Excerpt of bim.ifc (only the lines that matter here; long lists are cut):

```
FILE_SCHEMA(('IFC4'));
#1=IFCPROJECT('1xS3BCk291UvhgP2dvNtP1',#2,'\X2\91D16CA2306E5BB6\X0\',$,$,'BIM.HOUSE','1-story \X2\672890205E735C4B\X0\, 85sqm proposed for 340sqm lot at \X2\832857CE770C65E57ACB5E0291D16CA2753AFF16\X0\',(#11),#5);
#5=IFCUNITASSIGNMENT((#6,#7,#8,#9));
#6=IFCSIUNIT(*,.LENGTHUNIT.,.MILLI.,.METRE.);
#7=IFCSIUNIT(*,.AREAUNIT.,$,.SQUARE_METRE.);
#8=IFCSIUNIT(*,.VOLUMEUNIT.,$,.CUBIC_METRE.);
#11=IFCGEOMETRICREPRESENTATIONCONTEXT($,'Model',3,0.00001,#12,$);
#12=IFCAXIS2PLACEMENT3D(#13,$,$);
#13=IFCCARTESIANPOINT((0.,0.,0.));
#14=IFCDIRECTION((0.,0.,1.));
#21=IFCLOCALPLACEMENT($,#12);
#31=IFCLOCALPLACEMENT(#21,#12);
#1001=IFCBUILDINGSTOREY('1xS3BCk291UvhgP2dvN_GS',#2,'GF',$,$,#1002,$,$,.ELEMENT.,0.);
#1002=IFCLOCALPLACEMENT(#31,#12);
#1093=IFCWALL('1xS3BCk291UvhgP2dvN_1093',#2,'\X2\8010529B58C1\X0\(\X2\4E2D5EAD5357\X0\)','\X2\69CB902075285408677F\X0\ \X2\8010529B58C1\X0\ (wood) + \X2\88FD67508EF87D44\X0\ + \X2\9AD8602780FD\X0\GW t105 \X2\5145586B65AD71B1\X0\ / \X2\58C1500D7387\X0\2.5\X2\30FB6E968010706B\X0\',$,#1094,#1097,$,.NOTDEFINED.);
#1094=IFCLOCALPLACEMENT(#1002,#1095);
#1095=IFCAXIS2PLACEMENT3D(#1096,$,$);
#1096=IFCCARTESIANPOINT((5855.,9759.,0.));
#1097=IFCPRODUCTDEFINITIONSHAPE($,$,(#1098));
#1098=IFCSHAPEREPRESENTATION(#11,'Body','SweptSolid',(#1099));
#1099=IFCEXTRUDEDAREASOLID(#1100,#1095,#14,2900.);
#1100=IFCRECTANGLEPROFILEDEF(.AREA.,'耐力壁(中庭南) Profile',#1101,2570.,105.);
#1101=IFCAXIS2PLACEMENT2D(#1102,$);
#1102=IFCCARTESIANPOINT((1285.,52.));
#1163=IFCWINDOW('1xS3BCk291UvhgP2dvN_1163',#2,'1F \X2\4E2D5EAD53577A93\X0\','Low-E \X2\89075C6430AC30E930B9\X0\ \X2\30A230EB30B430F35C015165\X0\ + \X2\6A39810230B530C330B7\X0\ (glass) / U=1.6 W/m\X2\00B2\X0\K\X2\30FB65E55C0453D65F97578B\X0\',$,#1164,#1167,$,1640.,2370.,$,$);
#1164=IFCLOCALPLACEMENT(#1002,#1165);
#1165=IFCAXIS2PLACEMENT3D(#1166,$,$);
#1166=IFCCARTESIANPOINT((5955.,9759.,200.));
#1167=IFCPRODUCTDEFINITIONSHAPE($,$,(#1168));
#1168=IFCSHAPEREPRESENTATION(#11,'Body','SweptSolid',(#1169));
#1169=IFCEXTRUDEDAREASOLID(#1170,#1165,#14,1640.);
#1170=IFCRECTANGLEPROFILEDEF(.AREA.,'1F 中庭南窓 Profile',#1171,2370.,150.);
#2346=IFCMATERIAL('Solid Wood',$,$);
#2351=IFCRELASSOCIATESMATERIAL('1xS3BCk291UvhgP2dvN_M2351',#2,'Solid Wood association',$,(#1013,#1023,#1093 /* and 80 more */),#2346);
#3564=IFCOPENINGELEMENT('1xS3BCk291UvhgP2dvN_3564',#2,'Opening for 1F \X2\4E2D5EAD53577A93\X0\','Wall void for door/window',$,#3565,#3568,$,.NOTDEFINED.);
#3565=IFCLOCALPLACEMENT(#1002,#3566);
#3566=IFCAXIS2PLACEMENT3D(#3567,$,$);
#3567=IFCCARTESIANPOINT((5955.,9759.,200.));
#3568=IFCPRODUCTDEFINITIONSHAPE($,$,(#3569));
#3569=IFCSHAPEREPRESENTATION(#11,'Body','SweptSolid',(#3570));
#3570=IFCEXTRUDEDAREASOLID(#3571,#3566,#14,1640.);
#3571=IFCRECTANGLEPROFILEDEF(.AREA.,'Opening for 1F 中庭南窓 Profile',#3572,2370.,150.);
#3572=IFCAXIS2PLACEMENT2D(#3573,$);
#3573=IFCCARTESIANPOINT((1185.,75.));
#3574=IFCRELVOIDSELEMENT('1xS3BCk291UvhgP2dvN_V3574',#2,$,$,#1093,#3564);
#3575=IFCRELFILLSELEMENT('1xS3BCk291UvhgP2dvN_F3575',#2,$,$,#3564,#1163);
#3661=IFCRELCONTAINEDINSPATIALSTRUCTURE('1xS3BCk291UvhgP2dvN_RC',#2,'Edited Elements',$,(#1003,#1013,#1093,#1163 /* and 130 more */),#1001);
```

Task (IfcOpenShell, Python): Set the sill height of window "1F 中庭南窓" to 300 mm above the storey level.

```python
import numpy as np
import ifcopenshell
import ifcopenshell.api.geometry
import ifcopenshell.geom
import ifcopenshell.util.element
import ifcopenshell.util.placement
import ifcopenshell.util.shape
import ifcopenshell.util.unit

model = ifcopenshell.open("bim.ifc")
unit_scale = ifcopenshell.util.unit.calculate_unit_scale(model)

window = model.by_guid("1xS3BCk291UvhgP2dvN_1163")
opening = window.FillsVoids[0].RelatingOpeningElement
storey = ifcopenshell.util.element.get_container(window, ifc_class="IfcBuildingStorey")
level = ifcopenshell.util.placement.get_local_placement(storey.ObjectPlacement)[2, 3]

# The opening's origin need not be at the sill, so measure its lowest point.
shape = ifcopenshell.geom.create_shape(ifcopenshell.geom.settings(), opening)
bottom = ifcopenshell.util.shape.get_shape_bottom_elevation(shape, shape.geometry) / unit_scale
dz = level + 0.3 / unit_scale - bottom

shift = np.array([0.0, 0.0, dz])
# The window is not placed relative to its opening, so move both.
for product in (opening, window):
    matrix = ifcopenshell.util.placement.get_local_placement(product.ObjectPlacement)
    matrix[:3, 3] += shift
    ifcopenshell.api.geometry.edit_object_placement(model, product=product, matrix=matrix, is_si=False)

print(f"moved by {dz * unit_scale:+.3f} m")

model.write("bim_updated.ifc")
```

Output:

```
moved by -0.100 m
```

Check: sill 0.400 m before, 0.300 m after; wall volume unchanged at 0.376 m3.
